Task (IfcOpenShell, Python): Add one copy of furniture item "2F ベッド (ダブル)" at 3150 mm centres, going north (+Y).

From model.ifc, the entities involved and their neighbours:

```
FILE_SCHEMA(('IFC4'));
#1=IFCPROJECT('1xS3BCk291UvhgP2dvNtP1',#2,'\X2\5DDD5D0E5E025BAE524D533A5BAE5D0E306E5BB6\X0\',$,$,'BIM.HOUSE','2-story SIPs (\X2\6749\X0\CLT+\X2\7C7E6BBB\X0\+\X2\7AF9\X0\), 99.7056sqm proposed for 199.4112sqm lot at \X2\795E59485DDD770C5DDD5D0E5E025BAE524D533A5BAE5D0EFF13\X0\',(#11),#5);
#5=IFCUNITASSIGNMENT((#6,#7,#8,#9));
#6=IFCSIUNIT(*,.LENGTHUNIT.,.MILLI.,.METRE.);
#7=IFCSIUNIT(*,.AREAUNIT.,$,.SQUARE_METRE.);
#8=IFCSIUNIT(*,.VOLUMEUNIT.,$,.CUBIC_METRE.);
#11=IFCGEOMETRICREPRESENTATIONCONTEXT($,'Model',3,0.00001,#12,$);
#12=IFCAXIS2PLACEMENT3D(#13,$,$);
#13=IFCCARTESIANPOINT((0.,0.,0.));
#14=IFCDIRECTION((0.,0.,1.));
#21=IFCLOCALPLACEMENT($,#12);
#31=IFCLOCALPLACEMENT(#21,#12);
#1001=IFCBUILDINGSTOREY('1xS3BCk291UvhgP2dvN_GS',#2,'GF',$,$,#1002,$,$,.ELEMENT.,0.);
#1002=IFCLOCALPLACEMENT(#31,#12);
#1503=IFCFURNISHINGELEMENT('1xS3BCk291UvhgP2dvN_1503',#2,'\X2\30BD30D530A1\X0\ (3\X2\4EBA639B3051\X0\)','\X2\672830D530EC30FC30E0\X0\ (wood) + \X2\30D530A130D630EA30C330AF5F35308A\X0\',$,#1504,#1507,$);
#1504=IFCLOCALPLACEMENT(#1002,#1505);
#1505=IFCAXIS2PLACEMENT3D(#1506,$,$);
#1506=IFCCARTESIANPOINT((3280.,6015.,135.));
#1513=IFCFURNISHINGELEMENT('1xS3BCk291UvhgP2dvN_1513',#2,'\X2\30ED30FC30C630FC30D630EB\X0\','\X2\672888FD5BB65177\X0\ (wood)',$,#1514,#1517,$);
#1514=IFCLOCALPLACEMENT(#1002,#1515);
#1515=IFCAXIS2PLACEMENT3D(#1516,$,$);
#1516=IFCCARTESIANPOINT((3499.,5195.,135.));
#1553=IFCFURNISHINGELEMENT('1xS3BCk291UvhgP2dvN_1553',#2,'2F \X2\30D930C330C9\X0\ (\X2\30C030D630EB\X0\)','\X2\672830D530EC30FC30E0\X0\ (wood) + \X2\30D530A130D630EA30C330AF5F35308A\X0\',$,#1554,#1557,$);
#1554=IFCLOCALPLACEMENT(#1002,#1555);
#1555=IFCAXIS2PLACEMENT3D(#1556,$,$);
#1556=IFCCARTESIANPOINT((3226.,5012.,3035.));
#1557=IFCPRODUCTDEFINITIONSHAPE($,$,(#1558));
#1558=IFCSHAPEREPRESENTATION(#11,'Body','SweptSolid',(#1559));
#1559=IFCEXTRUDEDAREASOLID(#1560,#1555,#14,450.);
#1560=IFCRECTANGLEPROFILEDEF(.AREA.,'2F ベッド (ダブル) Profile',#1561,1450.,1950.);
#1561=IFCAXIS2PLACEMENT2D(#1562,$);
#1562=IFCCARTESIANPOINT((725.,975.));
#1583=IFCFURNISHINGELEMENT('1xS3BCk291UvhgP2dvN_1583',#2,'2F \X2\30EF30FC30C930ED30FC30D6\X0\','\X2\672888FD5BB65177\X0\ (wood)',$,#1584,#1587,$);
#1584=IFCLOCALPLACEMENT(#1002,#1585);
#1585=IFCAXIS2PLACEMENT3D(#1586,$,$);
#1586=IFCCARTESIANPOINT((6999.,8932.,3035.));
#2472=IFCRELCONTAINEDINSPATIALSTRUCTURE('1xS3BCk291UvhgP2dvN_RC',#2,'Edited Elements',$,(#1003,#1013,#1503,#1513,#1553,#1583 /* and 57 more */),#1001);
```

```python
import numpy as np
import ifcopenshell
import ifcopenshell.api.geometry
import ifcopenshell.api.root
import ifcopenshell.util.element
import ifcopenshell.util.placement
import ifcopenshell.util.unit

model = ifcopenshell.open("model.ifc")
unit_scale = ifcopenshell.util.unit.calculate_unit_scale(model)


def reuse_history(source, copy):
    """copy_class also copies each property set's owner history, people and application; keep the originals."""
    for rel in copy.IsDefinedBy:
        if rel.is_a("IfcRelDefinesByProperties") and (history := rel.RelatingPropertyDefinition.OwnerHistory):
            rel.RelatingPropertyDefinition.OwnerHistory = source.OwnerHistory
            ifcopenshell.util.element.remove_deep2(model, history)


source = model.by_id(1553)
base = ifcopenshell.util.placement.get_local_placement(source.ObjectPlacement)
step = np.array([0.0, 1.0, 0.0]) * 3.15 / unit_scale

for i in range(1, 2):
    copy = ifcopenshell.api.root.copy_class(model, product=source)
    copy.Representation = ifcopenshell.util.element.copy_deep(
        model, source.Representation, exclude=["IfcGeometricRepresentationContext", "IfcRepresentationMap"]
    )
    reuse_history(source, copy)
    matrix = base.copy()
    matrix[:3, 3] += i * step
    print("added at", matrix[:3, 3].round(3) + 0.0)
    ifcopenshell.api.geometry.edit_object_placement(model, product=copy, matrix=matrix, is_si=False)

model.write("model_rev.ifc")
```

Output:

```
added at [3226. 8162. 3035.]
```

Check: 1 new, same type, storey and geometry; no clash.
